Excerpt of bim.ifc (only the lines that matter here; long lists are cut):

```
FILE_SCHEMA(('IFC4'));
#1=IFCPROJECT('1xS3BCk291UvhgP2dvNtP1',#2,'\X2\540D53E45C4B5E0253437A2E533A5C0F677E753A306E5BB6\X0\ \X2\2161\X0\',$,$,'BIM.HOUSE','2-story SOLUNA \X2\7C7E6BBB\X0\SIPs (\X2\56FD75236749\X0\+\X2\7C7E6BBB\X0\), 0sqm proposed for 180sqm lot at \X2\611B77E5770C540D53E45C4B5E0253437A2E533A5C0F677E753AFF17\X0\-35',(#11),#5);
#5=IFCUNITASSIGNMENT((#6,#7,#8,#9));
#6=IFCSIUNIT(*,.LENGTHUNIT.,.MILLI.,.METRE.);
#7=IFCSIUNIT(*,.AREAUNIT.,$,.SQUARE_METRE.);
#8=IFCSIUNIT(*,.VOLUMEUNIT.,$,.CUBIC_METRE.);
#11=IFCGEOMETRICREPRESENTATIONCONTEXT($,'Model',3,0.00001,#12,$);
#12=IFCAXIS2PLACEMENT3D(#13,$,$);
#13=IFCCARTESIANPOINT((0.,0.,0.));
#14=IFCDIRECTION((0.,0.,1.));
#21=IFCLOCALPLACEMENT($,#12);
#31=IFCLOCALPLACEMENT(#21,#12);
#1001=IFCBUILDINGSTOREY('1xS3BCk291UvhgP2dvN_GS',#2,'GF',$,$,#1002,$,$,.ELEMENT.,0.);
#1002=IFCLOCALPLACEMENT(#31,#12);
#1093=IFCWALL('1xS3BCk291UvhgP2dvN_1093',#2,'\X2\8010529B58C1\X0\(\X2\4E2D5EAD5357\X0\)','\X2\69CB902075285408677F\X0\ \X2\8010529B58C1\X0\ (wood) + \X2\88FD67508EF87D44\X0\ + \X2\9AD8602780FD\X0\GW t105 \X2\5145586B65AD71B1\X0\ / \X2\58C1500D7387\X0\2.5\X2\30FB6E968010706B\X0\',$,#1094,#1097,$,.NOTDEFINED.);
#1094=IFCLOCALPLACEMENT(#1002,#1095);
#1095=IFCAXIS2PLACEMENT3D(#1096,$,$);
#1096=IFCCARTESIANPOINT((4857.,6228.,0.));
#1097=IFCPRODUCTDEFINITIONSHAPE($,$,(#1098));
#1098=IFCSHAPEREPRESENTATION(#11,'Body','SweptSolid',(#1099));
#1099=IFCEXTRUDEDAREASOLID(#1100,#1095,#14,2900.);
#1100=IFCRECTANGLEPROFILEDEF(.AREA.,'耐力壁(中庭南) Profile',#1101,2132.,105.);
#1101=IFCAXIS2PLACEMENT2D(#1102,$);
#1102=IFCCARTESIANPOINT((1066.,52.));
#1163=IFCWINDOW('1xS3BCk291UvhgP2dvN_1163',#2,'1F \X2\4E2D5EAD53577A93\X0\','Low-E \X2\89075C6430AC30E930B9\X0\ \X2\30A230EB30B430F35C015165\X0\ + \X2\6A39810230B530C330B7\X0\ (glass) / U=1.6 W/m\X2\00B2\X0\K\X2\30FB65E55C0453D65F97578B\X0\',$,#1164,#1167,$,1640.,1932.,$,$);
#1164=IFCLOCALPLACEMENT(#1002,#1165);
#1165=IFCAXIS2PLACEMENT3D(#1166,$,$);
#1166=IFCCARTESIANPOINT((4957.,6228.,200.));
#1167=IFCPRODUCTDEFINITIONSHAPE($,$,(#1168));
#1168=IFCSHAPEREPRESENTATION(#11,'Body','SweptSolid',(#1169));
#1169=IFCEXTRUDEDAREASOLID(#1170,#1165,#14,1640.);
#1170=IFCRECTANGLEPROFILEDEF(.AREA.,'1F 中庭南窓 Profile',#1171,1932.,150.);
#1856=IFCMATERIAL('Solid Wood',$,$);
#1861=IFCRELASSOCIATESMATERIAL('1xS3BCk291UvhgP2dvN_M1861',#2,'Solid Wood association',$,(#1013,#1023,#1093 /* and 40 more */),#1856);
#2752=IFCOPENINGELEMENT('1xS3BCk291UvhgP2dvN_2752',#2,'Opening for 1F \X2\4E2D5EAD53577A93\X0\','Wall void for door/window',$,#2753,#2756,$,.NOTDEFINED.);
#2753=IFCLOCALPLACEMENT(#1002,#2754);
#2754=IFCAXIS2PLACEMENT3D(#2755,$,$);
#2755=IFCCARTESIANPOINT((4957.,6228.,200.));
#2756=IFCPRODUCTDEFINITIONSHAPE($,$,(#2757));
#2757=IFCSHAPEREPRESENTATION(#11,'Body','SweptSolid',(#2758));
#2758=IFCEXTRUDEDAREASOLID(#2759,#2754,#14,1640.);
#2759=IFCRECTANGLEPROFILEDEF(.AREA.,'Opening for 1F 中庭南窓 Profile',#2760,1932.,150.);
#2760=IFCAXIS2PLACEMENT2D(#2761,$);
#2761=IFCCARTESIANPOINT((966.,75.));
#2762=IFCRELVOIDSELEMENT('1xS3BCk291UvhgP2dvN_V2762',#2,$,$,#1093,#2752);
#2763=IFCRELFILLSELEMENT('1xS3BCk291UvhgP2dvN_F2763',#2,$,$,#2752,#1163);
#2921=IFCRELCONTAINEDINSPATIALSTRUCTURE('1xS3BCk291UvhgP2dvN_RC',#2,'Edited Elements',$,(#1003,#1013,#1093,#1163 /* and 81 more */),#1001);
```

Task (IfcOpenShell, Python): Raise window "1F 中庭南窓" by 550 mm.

```python
import numpy as np
import ifcopenshell
import ifcopenshell.api.geometry
import ifcopenshell.util.placement
import ifcopenshell.util.unit

model = ifcopenshell.open("bim.ifc")
unit_scale = ifcopenshell.util.unit.calculate_unit_scale(model)

window = model.by_id(1163)
opening = window.FillsVoids[0].RelatingOpeningElement
dz = 0.55 / unit_scale

shift = np.array([0.0, 0.0, dz])
# The window is not placed relative to its opening, so move both.
for product in (opening, window):
    matrix = ifcopenshell.util.placement.get_local_placement(product.ObjectPlacement)
    matrix[:3, 3] += shift
    ifcopenshell.api.geometry.edit_object_placement(model, product=product, matrix=matrix, is_si=False)

print(f"moved by {dz * unit_scale:+.3f} m")

model.write("bim_edited.ifc")
```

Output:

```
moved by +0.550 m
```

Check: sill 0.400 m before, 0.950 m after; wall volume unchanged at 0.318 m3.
